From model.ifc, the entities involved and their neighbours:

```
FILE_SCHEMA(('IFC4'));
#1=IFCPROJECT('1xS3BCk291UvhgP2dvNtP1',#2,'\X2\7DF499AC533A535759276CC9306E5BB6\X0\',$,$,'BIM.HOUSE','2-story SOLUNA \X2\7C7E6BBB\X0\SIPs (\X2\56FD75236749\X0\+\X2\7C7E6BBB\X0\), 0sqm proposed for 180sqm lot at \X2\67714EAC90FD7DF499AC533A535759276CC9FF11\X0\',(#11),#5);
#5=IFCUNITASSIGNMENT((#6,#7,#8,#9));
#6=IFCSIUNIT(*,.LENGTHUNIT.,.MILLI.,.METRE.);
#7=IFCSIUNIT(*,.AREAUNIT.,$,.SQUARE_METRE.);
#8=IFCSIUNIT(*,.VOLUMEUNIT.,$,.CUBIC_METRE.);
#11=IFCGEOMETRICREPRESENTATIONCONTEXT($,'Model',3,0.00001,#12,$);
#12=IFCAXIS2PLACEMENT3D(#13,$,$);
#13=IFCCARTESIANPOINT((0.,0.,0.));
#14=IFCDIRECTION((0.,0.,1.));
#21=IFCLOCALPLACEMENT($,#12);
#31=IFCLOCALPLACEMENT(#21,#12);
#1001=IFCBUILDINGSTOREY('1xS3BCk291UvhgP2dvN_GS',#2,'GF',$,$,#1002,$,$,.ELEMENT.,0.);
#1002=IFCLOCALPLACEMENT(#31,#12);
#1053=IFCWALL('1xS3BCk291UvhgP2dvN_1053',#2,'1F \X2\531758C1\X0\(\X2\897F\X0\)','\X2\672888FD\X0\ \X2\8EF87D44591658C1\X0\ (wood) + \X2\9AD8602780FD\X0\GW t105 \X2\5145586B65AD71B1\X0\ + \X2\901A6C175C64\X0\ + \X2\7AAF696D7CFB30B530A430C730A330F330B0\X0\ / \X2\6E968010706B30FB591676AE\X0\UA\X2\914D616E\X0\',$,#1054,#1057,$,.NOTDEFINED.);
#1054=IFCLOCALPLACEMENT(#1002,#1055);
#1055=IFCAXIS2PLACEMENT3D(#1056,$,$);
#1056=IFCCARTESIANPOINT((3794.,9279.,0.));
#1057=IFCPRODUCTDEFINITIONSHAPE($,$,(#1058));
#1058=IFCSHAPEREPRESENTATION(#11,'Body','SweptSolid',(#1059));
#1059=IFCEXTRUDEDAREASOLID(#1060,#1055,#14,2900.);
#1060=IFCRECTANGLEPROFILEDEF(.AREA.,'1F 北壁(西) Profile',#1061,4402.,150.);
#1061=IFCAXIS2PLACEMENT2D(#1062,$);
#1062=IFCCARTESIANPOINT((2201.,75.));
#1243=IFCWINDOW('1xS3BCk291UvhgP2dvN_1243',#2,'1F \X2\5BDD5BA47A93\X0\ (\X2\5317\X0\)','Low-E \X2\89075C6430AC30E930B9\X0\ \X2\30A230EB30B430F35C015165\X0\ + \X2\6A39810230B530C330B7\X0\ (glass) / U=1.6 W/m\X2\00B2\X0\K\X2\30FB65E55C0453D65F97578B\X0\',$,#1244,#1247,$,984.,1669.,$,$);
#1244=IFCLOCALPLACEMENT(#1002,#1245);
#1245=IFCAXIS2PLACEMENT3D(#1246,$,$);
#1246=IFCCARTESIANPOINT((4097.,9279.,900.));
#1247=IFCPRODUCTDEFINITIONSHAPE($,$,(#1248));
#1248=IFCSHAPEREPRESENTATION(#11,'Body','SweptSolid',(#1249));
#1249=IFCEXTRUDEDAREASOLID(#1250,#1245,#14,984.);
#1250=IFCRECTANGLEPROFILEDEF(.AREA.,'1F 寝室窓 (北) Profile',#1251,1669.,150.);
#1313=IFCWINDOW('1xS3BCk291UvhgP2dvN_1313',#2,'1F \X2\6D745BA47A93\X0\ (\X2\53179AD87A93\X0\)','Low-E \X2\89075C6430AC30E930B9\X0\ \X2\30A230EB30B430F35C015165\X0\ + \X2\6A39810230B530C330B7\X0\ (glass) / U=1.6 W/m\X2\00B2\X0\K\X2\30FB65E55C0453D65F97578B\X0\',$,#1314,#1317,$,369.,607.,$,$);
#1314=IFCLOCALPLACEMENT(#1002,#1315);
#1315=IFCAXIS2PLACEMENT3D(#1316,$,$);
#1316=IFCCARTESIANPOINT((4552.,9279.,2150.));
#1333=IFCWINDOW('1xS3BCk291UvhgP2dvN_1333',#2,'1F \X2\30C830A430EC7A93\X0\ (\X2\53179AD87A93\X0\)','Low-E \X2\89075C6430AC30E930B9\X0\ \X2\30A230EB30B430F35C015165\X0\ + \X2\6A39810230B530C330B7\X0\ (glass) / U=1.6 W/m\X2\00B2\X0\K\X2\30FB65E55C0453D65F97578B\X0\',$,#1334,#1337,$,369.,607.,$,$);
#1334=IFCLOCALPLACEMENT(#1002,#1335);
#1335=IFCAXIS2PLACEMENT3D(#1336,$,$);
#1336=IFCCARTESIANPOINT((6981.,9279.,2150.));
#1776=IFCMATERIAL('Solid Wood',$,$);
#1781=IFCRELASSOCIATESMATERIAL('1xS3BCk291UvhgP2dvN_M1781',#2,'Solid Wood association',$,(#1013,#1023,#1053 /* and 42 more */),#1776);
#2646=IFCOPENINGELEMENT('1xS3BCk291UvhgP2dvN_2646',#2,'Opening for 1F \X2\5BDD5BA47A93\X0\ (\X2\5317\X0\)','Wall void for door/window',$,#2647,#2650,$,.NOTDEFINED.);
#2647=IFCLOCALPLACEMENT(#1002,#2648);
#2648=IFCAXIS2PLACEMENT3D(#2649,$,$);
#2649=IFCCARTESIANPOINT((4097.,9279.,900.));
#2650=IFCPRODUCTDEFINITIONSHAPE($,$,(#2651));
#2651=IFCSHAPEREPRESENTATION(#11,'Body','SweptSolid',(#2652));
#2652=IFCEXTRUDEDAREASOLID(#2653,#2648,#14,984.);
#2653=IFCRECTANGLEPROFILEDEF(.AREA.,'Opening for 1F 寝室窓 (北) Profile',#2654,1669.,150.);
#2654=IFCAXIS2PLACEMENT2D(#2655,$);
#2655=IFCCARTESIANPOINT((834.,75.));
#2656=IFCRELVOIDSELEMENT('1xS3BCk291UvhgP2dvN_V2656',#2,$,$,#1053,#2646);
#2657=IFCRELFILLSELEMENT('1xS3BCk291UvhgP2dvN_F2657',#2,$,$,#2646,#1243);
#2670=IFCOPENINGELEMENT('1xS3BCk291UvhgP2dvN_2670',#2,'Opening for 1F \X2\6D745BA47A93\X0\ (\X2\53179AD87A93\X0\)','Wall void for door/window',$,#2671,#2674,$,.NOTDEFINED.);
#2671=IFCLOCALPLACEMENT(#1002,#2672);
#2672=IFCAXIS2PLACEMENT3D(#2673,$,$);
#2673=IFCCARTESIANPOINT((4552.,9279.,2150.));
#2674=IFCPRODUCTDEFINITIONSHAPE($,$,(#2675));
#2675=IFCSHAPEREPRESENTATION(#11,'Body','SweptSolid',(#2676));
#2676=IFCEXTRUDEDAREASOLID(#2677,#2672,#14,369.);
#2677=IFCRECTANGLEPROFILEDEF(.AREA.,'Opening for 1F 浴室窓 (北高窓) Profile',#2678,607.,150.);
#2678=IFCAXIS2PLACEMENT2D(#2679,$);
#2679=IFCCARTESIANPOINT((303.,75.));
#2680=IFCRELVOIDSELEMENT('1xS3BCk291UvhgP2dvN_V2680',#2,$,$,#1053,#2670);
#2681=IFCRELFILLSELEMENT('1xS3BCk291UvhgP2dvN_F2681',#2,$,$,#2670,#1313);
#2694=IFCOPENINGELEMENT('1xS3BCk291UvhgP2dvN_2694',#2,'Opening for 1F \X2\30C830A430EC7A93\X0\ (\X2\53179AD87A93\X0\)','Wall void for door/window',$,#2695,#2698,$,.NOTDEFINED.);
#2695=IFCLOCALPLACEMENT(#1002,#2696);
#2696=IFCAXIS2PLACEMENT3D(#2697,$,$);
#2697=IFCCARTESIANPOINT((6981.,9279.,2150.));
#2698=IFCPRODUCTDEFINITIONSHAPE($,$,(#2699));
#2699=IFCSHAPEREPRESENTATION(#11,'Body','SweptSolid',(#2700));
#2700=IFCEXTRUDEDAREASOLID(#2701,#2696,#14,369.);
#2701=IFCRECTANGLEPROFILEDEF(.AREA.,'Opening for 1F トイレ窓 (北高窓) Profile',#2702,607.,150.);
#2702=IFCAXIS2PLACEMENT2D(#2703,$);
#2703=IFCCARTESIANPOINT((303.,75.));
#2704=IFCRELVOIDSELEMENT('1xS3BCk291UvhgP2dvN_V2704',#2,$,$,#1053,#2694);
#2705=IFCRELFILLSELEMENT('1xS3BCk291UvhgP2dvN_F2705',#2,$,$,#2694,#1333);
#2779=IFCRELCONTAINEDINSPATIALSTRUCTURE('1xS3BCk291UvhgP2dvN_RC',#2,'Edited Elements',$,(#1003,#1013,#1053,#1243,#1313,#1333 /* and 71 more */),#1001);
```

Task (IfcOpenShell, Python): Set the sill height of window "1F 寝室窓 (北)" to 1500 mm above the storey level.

```python
import numpy as np
import ifcopenshell
import ifcopenshell.api.geometry
import ifcopenshell.geom
import ifcopenshell.util.element
import ifcopenshell.util.placement
import ifcopenshell.util.shape
import ifcopenshell.util.unit

model = ifcopenshell.open("model.ifc")
unit_scale = ifcopenshell.util.unit.calculate_unit_scale(model)

window = model.by_id(1243)
opening = window.FillsVoids[0].RelatingOpeningElement
storey = ifcopenshell.util.element.get_container(window, ifc_class="IfcBuildingStorey")
level = ifcopenshell.util.placement.get_local_placement(storey.ObjectPlacement)[2, 3]

# The opening's origin need not be at the sill, so measure its lowest point.
shape = ifcopenshell.geom.create_shape(ifcopenshell.geom.settings(), opening)
bottom = ifcopenshell.util.shape.get_shape_bottom_elevation(shape, shape.geometry) / unit_scale
dz = level + 1500.0 - bottom

shift = np.array([0.0, 0.0, dz])
# The window is not placed relative to its opening, so move both.
for product in (opening, window):
    matrix = ifcopenshell.util.placement.get_local_placement(product.ObjectPlacement)
    matrix[:3, 3] += shift
    ifcopenshell.api.geometry.edit_object_placement(model, product=product, matrix=matrix, is_si=False)

print(f"moved by {dz * unit_scale:+.3f} m")

model.write("model_updated.ifc")
```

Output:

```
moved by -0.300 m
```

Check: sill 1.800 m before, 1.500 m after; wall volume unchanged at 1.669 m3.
